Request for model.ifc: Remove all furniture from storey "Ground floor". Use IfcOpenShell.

First a look at what the model holds.

```python
import ifcopenshell
import ifcopenshell.util.element

model = ifcopenshell.open("model.ifc")
print(model.schema)
storey = next(s for s in model.by_type("IfcBuildingStorey") if s.Name == "Ground floor")
furniture = [e for e in ifcopenshell.util.element.get_decomposition(storey) if e.is_a("IfcFurnishingElement")]
seen = {}
for e in furniture:
    element_type = ifcopenshell.util.element.get_type(e)
    name = element_type.Name if element_type not in (None, e) else None
    seen[name] = seen.get(name, 0) + 1
for name, count in sorted(seen.items(), key=str):
    print(count, "x", name)
```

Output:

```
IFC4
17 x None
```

```python
import ifcopenshell
import ifcopenshell.api.root
import ifcopenshell.util.element

model = ifcopenshell.open("model.ifc")

storey = next(s for s in model.by_type("IfcBuildingStorey") if s.Name == "Ground floor")
furniture = [e for e in ifcopenshell.util.element.get_decomposition(storey) if e.is_a("IfcFurnishingElement")]

for e in furniture:
    ifcopenshell.api.root.remove_product(model, product=e)
print(len(furniture), "removed")

model.write("model_edited.ifc")
```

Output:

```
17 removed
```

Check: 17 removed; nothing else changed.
